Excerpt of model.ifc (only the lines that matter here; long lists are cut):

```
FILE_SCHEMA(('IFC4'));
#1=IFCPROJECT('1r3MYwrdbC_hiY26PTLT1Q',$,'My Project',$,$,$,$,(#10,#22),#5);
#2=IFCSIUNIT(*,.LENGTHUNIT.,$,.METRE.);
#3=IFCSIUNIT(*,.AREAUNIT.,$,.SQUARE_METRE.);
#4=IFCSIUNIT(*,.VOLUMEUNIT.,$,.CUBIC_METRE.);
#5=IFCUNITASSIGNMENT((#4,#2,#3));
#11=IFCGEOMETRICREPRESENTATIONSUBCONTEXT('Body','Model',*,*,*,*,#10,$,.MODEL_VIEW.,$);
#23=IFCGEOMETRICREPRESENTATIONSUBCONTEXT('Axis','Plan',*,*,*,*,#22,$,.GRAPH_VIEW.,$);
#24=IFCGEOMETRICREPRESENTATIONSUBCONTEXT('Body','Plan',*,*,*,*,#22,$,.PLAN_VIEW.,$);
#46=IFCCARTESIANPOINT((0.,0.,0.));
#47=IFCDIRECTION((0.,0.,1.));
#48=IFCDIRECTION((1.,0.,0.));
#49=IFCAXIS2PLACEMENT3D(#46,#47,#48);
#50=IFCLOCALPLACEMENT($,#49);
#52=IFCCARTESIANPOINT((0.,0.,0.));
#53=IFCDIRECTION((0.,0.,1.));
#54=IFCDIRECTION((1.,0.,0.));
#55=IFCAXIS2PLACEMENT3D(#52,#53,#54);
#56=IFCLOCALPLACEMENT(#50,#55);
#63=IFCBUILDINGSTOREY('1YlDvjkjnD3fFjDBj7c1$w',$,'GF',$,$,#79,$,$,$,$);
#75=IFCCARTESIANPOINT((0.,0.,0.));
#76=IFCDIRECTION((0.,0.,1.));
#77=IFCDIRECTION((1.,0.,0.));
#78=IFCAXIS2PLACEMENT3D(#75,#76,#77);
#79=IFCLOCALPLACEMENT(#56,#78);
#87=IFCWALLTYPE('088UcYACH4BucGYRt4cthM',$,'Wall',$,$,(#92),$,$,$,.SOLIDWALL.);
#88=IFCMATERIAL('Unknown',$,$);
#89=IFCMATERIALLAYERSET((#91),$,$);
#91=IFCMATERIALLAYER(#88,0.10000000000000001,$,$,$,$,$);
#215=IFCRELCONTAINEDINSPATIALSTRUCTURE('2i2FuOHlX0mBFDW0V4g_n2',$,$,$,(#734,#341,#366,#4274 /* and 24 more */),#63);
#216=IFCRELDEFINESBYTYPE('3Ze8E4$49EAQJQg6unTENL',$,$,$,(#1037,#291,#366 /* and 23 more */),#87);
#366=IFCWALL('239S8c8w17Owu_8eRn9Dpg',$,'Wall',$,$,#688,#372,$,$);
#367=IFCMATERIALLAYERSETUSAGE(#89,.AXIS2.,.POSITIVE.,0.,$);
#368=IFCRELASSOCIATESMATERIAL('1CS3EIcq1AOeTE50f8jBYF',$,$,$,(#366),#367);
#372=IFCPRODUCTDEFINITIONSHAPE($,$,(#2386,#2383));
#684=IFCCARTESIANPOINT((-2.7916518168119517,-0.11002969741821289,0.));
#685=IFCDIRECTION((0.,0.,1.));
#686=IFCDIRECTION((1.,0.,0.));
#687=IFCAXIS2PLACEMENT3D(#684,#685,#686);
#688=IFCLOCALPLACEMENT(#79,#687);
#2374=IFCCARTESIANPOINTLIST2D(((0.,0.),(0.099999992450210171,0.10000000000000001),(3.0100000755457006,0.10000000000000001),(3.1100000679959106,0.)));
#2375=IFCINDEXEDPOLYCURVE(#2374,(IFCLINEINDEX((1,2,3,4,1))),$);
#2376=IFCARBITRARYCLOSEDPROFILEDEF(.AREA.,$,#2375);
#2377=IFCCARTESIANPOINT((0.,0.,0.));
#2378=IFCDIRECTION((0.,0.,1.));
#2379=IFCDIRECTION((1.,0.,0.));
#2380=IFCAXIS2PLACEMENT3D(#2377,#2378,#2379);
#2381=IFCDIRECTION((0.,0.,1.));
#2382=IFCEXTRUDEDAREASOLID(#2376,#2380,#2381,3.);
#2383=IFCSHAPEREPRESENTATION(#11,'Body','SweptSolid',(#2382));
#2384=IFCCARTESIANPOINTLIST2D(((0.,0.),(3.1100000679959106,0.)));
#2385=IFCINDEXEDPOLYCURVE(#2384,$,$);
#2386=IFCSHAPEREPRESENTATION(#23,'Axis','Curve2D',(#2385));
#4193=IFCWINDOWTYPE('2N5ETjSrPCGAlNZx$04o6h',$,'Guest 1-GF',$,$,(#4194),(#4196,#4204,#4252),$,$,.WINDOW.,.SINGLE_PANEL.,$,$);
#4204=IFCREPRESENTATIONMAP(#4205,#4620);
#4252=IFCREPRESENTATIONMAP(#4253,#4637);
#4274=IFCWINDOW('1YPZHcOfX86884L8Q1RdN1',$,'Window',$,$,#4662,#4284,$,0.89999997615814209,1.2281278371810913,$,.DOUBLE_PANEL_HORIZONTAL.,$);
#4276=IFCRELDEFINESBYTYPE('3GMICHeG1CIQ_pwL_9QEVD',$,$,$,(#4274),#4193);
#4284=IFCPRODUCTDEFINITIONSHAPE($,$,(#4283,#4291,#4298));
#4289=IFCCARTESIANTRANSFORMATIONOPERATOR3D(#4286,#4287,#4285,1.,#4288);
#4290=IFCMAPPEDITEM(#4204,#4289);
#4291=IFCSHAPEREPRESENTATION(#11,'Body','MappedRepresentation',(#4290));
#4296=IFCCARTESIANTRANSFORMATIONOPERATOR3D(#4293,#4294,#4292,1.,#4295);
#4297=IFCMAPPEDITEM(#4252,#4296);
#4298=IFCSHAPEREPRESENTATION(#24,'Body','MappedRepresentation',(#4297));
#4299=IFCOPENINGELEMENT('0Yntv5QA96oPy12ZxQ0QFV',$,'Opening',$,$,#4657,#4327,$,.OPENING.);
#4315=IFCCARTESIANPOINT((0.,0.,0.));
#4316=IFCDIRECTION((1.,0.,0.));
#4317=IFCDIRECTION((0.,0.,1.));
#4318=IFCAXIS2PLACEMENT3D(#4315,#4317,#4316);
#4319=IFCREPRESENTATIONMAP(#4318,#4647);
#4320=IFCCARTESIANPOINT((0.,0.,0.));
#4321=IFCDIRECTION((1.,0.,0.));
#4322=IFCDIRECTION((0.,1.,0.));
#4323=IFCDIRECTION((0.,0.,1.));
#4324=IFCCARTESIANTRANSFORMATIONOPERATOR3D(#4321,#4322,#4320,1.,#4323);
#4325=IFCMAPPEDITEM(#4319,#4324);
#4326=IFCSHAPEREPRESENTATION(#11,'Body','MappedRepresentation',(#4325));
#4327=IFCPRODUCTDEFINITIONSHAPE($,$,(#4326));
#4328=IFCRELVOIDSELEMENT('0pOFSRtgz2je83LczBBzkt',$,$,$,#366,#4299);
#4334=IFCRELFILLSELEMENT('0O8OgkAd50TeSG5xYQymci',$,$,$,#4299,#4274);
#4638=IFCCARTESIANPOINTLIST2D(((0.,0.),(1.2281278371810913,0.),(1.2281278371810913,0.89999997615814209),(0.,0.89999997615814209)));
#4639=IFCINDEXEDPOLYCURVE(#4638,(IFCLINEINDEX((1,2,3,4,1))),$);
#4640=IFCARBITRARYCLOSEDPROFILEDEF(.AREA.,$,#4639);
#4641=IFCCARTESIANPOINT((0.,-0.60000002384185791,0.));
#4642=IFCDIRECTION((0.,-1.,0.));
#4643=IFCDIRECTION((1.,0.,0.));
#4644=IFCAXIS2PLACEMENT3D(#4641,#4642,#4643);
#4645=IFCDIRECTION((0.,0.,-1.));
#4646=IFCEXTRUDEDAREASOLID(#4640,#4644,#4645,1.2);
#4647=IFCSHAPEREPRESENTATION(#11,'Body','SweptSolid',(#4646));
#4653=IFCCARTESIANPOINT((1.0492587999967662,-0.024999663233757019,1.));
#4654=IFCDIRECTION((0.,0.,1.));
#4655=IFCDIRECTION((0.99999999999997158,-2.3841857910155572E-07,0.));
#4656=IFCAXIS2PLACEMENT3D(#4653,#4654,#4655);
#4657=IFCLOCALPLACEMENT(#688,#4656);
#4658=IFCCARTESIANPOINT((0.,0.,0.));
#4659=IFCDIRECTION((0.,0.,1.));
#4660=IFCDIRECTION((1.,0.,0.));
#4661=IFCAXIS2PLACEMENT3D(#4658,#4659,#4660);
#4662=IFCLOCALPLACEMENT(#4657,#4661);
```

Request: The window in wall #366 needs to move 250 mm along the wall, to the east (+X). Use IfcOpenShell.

```python
import ifcopenshell
import ifcopenshell.api.geometry
import ifcopenshell.util.placement

model = ifcopenshell.open("model.ifc")

window = model.by_guid("1YPZHcOfX86884L8Q1RdN1")
opening = window.FillsVoids[0].RelatingOpeningElement
wall = opening.VoidsElements[0].RelatingBuildingElement

wall_matrix = ifcopenshell.util.placement.get_local_placement(wall.ObjectPlacement)
shift = wall_matrix[:3, 0] * 0.25
before = ifcopenshell.util.placement.get_local_placement(window.ObjectPlacement)[:3, 3].copy()

# The window is placed relative to its opening, so it follows when the opening moves.
matrix = ifcopenshell.util.placement.get_local_placement(opening.ObjectPlacement)
matrix[:3, 3] += shift
ifcopenshell.api.geometry.edit_object_placement(
    model, product=opening, matrix=matrix, is_si=False, should_transform_children=True
)

after = ifcopenshell.util.placement.get_local_placement(window.ObjectPlacement)[:3, 3]
print("window moved by", (after - before).round(3) + 0.0)

model.write("model_edited.ifc")
```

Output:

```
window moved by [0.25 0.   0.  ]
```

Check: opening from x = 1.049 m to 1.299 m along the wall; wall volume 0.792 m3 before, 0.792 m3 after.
